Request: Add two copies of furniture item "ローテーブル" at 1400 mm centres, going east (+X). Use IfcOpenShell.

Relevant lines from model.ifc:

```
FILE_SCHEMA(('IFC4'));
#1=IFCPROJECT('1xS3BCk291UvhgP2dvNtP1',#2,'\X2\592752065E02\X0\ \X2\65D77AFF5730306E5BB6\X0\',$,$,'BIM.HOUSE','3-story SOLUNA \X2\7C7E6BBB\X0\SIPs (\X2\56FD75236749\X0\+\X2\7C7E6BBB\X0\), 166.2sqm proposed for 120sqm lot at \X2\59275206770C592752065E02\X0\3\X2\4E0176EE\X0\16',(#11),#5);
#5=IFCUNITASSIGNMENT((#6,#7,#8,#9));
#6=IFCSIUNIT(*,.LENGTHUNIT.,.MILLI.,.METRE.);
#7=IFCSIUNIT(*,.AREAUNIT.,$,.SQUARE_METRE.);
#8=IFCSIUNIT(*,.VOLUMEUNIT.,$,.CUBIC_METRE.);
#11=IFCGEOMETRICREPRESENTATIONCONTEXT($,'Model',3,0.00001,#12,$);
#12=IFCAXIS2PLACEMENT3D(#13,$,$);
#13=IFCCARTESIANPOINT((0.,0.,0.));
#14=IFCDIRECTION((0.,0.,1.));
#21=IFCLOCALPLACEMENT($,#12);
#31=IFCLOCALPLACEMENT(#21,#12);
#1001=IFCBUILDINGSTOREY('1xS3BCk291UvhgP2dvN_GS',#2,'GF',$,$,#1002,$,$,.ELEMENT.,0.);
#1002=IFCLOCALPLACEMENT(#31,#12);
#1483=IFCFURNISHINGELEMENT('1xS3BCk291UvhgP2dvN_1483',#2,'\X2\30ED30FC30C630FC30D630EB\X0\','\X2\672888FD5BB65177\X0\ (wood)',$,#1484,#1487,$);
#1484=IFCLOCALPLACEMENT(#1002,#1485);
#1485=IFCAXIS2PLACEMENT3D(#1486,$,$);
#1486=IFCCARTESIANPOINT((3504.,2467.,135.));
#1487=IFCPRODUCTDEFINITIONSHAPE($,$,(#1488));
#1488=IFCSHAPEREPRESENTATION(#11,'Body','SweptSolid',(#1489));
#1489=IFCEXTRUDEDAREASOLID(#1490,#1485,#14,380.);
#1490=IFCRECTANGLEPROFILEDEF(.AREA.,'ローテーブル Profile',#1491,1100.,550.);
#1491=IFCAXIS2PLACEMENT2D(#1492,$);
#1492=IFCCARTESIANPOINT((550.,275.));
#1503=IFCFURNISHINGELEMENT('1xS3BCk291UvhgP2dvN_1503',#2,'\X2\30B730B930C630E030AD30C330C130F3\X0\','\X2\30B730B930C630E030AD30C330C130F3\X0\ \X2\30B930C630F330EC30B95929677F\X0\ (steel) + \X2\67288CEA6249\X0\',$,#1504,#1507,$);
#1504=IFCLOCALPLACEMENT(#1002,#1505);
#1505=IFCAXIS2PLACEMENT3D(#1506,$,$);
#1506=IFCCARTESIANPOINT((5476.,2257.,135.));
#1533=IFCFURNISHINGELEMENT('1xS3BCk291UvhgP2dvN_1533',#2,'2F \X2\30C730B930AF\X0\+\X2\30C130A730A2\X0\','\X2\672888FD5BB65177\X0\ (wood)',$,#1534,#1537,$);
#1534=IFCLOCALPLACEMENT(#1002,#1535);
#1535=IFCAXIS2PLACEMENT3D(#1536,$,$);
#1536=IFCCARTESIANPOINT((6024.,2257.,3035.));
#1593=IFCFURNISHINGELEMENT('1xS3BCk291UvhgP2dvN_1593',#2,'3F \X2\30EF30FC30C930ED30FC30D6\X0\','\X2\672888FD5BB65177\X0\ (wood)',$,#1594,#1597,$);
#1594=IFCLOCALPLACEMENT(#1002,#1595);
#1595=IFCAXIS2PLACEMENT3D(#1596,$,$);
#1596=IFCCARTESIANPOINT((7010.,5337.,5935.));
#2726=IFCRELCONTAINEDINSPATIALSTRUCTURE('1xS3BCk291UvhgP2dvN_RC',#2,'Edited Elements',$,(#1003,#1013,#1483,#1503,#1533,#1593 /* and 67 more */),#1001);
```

```python
import numpy as np
import ifcopenshell
import ifcopenshell.api.geometry
import ifcopenshell.api.root
import ifcopenshell.util.element
import ifcopenshell.util.placement
import ifcopenshell.util.unit

model = ifcopenshell.open("model.ifc")
unit_scale = ifcopenshell.util.unit.calculate_unit_scale(model)


def reuse_history(source, copy):
    """copy_class also copies each property set's owner history, people and application; keep the originals."""
    for rel in copy.IsDefinedBy:
        if rel.is_a("IfcRelDefinesByProperties") and (history := rel.RelatingPropertyDefinition.OwnerHistory):
            rel.RelatingPropertyDefinition.OwnerHistory = source.OwnerHistory
            ifcopenshell.util.element.remove_deep2(model, history)


source = model.by_guid("1xS3BCk291UvhgP2dvN_1483")
base = ifcopenshell.util.placement.get_local_placement(source.ObjectPlacement)
step = np.array([1.0, 0.0, 0.0]) * 1.4 / unit_scale

for i in range(1, 3):
    copy = ifcopenshell.api.root.copy_class(model, product=source)
    copy.Representation = ifcopenshell.util.element.copy_deep(
        model, source.Representation, exclude=["IfcGeometricRepresentationContext", "IfcRepresentationMap"]
    )
    reuse_history(source, copy)
    matrix = base.copy()
    matrix[:3, 3] += i * step
    print("added at", matrix[:3, 3].round(3) + 0.0)
    ifcopenshell.api.geometry.edit_object_placement(model, product=copy, matrix=matrix, is_si=False)

model.write("model_updated.ifc")
```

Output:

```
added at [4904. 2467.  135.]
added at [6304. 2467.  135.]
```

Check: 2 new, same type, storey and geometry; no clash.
